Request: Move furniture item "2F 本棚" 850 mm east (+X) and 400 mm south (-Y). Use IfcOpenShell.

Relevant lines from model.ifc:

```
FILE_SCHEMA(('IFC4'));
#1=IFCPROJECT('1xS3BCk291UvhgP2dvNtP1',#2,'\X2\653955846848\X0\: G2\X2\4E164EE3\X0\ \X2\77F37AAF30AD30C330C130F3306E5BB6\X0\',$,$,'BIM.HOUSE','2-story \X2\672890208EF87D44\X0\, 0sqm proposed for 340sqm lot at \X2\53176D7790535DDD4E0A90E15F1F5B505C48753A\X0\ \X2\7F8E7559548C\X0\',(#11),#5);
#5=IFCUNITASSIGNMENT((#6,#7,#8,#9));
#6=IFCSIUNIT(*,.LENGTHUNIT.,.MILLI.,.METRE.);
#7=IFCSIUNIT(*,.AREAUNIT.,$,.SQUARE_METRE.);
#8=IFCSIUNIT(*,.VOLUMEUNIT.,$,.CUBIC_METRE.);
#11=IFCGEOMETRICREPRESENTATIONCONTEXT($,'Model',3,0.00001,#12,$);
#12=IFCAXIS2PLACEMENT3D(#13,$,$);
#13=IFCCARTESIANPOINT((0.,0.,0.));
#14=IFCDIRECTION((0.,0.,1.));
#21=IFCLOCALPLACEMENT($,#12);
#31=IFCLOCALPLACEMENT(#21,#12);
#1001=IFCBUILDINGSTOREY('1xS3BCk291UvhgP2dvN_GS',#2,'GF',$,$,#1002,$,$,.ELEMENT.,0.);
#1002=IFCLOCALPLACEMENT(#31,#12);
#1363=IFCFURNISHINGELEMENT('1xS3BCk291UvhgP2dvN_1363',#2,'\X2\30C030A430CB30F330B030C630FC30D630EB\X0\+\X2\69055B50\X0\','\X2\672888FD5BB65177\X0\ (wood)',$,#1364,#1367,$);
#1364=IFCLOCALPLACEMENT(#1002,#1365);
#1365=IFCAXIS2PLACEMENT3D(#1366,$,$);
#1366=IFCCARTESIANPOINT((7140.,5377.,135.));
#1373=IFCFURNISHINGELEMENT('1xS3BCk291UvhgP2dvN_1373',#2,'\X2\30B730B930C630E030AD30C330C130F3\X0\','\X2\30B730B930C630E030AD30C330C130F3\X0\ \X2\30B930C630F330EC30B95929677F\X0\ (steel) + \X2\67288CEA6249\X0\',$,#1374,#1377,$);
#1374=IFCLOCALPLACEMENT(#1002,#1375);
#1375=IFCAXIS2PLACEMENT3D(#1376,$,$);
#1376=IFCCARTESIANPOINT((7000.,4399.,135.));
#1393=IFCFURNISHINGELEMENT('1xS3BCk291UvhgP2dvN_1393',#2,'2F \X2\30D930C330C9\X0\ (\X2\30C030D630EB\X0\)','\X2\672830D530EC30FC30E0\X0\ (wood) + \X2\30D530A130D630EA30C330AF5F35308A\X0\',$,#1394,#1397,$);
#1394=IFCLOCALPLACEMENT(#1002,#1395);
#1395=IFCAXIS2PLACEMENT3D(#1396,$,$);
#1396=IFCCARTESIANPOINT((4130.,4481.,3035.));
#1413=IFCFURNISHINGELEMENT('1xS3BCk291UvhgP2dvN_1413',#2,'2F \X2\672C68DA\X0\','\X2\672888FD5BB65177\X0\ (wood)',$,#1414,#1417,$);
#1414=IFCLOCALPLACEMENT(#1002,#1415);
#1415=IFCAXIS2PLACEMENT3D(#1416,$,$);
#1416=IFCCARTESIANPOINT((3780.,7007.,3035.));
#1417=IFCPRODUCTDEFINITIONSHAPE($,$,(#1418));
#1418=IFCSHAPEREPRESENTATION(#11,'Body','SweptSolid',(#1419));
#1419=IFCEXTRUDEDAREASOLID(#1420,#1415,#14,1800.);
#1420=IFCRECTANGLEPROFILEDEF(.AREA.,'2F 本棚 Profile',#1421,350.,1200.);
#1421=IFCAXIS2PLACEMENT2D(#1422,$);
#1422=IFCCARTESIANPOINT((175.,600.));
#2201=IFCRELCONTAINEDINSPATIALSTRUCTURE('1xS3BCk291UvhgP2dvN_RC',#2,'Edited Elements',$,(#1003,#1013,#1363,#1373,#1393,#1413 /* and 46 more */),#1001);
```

```python
import ifcopenshell
import ifcopenshell.api.geometry
import ifcopenshell.util.placement

model = ifcopenshell.open("model.ifc")

item = model.by_guid("1xS3BCk291UvhgP2dvN_1413")
matrix = ifcopenshell.util.placement.get_local_placement(item.ObjectPlacement)
matrix[0, 3] += 850.0
matrix[1, 3] -= 400.0
ifcopenshell.api.geometry.edit_object_placement(model, product=item, matrix=matrix, is_si=False)

print(ifcopenshell.util.placement.get_local_placement(item.ObjectPlacement).round(3) + 0.0)

model.write("model_rev.ifc")
```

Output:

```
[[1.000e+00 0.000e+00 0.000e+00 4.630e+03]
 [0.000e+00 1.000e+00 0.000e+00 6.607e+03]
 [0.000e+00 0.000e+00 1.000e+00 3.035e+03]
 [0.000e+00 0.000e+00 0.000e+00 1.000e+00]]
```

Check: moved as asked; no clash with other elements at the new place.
